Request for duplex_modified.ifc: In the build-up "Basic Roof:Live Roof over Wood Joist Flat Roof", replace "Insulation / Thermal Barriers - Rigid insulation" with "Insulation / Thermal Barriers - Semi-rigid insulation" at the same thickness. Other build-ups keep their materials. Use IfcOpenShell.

First a look at what the model holds.

```python
import ifcopenshell
import ifcopenshell.util.element

model = ifcopenshell.open("duplex_modified.ifc")
print(model.schema)
for layer_set in model.by_type("IfcMaterialLayerSet"):
    if layer_set.LayerSetName == "Basic Roof:Live Roof over Wood Joist Flat Roof":
        for layer in layer_set.MaterialLayers:
            print(layer.id(), layer.Material and layer.Material.Name, layer.LayerThickness, sep=" | ")
        print(len(ifcopenshell.util.element.get_elements_by_material(model, layer_set)), "elements and types use it")
print(sorted(m.Name for m in model.by_type("IfcMaterial") if m.Name)[:60])
```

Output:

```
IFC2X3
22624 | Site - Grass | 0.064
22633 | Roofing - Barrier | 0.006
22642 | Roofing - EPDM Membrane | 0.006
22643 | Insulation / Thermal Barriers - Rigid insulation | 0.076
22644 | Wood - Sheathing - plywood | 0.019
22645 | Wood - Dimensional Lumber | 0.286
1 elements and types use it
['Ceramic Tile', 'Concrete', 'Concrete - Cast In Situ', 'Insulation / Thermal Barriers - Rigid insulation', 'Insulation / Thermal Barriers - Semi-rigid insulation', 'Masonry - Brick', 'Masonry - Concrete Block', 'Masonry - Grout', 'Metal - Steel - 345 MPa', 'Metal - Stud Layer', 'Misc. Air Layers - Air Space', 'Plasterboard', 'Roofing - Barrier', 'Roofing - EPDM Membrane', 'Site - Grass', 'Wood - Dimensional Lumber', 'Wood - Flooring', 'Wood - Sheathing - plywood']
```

```python
import ifcopenshell
import ifcopenshell.api.material

model = ifcopenshell.open("duplex_modified.ifc")

layer_set = next(s for s in model.by_type("IfcMaterialLayerSet") if s.LayerSetName == "Basic Roof:Live Roof over Wood Joist Flat Roof")
layer = next(l for l in layer_set.MaterialLayers if l.Material and l.Material.Name == "Insulation / Thermal Barriers - Rigid insulation")
material = next(m for m in model.by_type("IfcMaterial") if m.Name == "Insulation / Thermal Barriers - Semi-rigid insulation")

# Point this one layer at the other material; renaming the old one would change it everywhere.
ifcopenshell.api.material.edit_layer(model, layer=layer, attributes={}, material=material)

print([l.Material.Name if l.Material else None for l in layer_set.MaterialLayers])

model.write("duplex_modified_rev.ifc")
```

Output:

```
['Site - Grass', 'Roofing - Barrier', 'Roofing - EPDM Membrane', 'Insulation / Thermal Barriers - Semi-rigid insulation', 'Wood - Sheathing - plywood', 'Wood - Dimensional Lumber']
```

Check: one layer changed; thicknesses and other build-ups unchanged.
